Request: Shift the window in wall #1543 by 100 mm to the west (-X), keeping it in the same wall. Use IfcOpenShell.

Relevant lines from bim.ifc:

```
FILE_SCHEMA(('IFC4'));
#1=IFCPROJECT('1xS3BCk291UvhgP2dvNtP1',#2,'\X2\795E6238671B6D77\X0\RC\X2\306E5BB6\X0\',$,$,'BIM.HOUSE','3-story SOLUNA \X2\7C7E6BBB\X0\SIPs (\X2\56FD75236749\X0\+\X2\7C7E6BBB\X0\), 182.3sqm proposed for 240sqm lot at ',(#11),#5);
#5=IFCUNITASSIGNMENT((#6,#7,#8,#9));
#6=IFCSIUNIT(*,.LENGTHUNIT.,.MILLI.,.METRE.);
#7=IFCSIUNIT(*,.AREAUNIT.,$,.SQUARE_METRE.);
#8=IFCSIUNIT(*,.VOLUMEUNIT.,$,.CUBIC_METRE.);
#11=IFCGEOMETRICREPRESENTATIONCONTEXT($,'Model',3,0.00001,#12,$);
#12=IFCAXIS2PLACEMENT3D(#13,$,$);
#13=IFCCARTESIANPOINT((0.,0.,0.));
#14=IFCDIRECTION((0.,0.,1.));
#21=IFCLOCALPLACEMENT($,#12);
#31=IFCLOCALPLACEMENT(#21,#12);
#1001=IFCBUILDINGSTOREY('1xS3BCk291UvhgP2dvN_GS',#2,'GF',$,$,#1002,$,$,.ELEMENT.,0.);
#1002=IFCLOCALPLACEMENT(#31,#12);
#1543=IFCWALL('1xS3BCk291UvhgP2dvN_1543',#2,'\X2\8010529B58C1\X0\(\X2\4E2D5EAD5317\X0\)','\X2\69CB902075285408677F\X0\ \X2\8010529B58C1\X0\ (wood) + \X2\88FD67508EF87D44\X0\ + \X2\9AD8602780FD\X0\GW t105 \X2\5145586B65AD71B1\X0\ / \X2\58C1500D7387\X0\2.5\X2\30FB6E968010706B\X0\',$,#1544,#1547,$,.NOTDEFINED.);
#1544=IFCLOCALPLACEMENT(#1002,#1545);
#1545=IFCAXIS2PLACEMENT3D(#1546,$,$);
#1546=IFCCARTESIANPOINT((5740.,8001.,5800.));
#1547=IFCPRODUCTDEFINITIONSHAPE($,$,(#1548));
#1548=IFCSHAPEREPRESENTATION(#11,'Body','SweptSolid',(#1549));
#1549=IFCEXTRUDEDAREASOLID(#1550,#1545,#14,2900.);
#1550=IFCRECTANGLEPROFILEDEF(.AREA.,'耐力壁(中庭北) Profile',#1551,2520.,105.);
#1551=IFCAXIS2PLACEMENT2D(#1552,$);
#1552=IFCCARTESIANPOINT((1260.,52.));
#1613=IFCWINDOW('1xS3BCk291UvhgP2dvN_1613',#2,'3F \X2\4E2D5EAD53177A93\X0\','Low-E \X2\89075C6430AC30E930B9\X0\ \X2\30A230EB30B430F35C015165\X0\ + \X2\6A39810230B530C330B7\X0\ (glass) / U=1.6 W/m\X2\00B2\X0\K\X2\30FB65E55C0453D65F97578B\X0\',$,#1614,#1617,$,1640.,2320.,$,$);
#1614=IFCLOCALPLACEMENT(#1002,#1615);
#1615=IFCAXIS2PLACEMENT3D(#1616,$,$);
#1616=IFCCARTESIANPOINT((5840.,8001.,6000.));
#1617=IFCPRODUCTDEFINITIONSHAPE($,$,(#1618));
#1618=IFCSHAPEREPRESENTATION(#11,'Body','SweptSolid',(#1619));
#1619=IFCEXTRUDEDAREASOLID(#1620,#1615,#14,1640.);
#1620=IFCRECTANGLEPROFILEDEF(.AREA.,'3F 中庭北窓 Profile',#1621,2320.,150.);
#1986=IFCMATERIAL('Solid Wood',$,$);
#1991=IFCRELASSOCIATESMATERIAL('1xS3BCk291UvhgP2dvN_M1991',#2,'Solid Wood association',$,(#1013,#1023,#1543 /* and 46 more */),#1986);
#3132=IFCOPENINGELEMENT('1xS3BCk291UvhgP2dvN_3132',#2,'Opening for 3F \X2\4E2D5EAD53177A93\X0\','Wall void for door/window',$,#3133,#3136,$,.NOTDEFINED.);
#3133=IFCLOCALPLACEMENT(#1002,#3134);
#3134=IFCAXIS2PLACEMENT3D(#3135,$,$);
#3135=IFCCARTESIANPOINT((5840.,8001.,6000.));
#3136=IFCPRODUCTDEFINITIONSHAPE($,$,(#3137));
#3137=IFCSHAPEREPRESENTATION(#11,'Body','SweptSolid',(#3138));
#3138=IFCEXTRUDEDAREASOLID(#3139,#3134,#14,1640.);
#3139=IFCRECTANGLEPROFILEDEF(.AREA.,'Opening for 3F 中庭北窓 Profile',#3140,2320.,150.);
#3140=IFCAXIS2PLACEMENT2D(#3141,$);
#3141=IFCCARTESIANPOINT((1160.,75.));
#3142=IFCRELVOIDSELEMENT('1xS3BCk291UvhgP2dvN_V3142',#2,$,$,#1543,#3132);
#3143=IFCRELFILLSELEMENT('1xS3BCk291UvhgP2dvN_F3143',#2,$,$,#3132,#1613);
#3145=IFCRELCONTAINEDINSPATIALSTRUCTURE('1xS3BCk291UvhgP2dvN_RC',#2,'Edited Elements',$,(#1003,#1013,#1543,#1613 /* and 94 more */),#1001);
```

```python
import ifcopenshell
import ifcopenshell.api.geometry
import ifcopenshell.util.placement

model = ifcopenshell.open("bim.ifc")

window = model.by_id(1613)
opening = window.FillsVoids[0].RelatingOpeningElement
wall = opening.VoidsElements[0].RelatingBuildingElement

wall_matrix = ifcopenshell.util.placement.get_local_placement(wall.ObjectPlacement)
shift = wall_matrix[:3, 0] * -100.0
before = ifcopenshell.util.placement.get_local_placement(window.ObjectPlacement)[:3, 3].copy()

# The window is not placed relative to its opening, so move both.
for product in (opening, window):
    matrix = ifcopenshell.util.placement.get_local_placement(product.ObjectPlacement)
    matrix[:3, 3] += shift
    ifcopenshell.api.geometry.edit_object_placement(model, product=product, matrix=matrix, is_si=False)

after = ifcopenshell.util.placement.get_local_placement(window.ObjectPlacement)[:3, 3]
print("window moved by", (after - before).round(3) + 0.0)

model.write("bim_updated.ifc")
```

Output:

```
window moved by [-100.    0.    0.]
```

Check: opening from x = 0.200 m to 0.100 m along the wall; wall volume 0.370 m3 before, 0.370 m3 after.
